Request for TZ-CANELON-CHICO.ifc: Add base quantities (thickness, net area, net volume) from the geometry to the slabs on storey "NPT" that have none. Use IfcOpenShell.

First a look at what the model holds.

```python
import ifcopenshell
import ifcopenshell.util.element
import ifcopenshell.util.unit

model = ifcopenshell.open("TZ-CANELON-CHICO.ifc")
print(model.schema)
for unit_type in ("LENGTHUNIT", "AREAUNIT", "VOLUMEUNIT"):
    print(unit_type, ifcopenshell.util.unit.calculate_unit_scale(model, unit_type))
storey = next(s for s in model.by_type("IfcBuildingStorey") if s.Name == "NPT")
slabs = [e for e in ifcopenshell.util.element.get_decomposition(storey) if e.is_a("IfcSlab")]
for e in sorted(slabs, key=lambda e: e.id()):
    print(e.id(), e.is_a(), e.Name, list(ifcopenshell.util.element.get_psets(e, qtos_only=True)), sep=" | ")
```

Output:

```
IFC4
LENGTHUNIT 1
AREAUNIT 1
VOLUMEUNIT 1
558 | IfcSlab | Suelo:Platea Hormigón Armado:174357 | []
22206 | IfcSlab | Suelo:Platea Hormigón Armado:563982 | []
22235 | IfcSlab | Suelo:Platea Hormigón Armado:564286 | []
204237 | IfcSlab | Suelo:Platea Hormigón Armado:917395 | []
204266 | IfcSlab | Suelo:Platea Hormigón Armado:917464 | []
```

```python
import ifcopenshell
import ifcopenshell.api.pset
import ifcopenshell.geom
import ifcopenshell.util.element
import ifcopenshell.util.shape
import ifcopenshell.util.unit

model = ifcopenshell.open("TZ-CANELON-CHICO.ifc")
unit_scale = ifcopenshell.util.unit.calculate_unit_scale(model)
area_scale = ifcopenshell.util.unit.calculate_unit_scale(model, "AREAUNIT")
volume_scale = ifcopenshell.util.unit.calculate_unit_scale(model, "VOLUMEUNIT")
settings = ifcopenshell.geom.settings()

storey = next(s for s in model.by_type("IfcBuildingStorey") if s.Name == "NPT")
slabs = [e for e in ifcopenshell.util.element.get_decomposition(storey) if e.is_a("IfcSlab")]

for e in sorted(slabs, key=lambda e: e.id()):
    if ifcopenshell.util.element.get_psets(e, qtos_only=True, should_inherit=False):
        continue
    # Geometry comes back in metres, in the element's own axes.
    shape = ifcopenshell.geom.create_shape(settings, e)
    values = {
        "Width": ifcopenshell.util.shape.get_z(shape.geometry) / unit_scale,
        "NetArea": ifcopenshell.util.shape.get_footprint_area(shape.geometry) / area_scale,
        "NetVolume": ifcopenshell.util.shape.get_volume(shape.geometry) / volume_scale,
    }
    qto = ifcopenshell.api.pset.add_qto(model, product=e, name="Qto_SlabBaseQuantities")
    ifcopenshell.api.pset.edit_qto(model, qto=qto, properties=values)
    print(e.id(), {k: round(v, 3) for k, v in values.items()})

model.write("TZ-CANELON-CHICO_updated.ifc")
```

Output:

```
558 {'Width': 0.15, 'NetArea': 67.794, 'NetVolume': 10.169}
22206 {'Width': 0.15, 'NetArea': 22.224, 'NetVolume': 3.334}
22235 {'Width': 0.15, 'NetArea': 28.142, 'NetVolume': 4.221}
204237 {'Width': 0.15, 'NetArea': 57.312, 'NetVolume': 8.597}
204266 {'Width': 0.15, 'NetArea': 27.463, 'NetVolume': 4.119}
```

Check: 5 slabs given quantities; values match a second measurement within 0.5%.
